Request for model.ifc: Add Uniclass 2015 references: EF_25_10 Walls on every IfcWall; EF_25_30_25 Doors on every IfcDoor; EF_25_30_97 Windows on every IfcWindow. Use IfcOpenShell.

First a look at what the model holds.

```python
import ifcopenshell

model = ifcopenshell.open("model.ifc")
print(model.schema)
print("classifications:", [c.Name for c in model.by_type("IfcClassification")])
for ifc_class in ("IfcDoor", "IfcRoof", "IfcStair", "IfcWall", "IfcWindow"):
    print(ifc_class, len(model.by_type(ifc_class)))
```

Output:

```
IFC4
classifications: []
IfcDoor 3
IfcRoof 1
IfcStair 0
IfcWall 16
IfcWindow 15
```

```python
import ifcopenshell
import ifcopenshell.api.classification

model = ifcopenshell.open("model.ifc")

system = ifcopenshell.api.classification.add_classification(model, classification="Uniclass 2015")

codes = {
    "IfcWall": ("EF_25_10", "Walls"),
    "IfcDoor": ("EF_25_30_25", "Doors"),
    "IfcWindow": ("EF_25_30_97", "Windows"),
}
for ifc_class, (code, name) in codes.items():
    products = model.by_type(ifc_class)
    ifcopenshell.api.classification.add_reference(
        model, products=products, classification=system, identification=code, name=name
    )
    print(code, len(products))

model.write("model_updated.ifc")
```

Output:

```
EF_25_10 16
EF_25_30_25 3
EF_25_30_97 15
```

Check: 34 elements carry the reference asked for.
